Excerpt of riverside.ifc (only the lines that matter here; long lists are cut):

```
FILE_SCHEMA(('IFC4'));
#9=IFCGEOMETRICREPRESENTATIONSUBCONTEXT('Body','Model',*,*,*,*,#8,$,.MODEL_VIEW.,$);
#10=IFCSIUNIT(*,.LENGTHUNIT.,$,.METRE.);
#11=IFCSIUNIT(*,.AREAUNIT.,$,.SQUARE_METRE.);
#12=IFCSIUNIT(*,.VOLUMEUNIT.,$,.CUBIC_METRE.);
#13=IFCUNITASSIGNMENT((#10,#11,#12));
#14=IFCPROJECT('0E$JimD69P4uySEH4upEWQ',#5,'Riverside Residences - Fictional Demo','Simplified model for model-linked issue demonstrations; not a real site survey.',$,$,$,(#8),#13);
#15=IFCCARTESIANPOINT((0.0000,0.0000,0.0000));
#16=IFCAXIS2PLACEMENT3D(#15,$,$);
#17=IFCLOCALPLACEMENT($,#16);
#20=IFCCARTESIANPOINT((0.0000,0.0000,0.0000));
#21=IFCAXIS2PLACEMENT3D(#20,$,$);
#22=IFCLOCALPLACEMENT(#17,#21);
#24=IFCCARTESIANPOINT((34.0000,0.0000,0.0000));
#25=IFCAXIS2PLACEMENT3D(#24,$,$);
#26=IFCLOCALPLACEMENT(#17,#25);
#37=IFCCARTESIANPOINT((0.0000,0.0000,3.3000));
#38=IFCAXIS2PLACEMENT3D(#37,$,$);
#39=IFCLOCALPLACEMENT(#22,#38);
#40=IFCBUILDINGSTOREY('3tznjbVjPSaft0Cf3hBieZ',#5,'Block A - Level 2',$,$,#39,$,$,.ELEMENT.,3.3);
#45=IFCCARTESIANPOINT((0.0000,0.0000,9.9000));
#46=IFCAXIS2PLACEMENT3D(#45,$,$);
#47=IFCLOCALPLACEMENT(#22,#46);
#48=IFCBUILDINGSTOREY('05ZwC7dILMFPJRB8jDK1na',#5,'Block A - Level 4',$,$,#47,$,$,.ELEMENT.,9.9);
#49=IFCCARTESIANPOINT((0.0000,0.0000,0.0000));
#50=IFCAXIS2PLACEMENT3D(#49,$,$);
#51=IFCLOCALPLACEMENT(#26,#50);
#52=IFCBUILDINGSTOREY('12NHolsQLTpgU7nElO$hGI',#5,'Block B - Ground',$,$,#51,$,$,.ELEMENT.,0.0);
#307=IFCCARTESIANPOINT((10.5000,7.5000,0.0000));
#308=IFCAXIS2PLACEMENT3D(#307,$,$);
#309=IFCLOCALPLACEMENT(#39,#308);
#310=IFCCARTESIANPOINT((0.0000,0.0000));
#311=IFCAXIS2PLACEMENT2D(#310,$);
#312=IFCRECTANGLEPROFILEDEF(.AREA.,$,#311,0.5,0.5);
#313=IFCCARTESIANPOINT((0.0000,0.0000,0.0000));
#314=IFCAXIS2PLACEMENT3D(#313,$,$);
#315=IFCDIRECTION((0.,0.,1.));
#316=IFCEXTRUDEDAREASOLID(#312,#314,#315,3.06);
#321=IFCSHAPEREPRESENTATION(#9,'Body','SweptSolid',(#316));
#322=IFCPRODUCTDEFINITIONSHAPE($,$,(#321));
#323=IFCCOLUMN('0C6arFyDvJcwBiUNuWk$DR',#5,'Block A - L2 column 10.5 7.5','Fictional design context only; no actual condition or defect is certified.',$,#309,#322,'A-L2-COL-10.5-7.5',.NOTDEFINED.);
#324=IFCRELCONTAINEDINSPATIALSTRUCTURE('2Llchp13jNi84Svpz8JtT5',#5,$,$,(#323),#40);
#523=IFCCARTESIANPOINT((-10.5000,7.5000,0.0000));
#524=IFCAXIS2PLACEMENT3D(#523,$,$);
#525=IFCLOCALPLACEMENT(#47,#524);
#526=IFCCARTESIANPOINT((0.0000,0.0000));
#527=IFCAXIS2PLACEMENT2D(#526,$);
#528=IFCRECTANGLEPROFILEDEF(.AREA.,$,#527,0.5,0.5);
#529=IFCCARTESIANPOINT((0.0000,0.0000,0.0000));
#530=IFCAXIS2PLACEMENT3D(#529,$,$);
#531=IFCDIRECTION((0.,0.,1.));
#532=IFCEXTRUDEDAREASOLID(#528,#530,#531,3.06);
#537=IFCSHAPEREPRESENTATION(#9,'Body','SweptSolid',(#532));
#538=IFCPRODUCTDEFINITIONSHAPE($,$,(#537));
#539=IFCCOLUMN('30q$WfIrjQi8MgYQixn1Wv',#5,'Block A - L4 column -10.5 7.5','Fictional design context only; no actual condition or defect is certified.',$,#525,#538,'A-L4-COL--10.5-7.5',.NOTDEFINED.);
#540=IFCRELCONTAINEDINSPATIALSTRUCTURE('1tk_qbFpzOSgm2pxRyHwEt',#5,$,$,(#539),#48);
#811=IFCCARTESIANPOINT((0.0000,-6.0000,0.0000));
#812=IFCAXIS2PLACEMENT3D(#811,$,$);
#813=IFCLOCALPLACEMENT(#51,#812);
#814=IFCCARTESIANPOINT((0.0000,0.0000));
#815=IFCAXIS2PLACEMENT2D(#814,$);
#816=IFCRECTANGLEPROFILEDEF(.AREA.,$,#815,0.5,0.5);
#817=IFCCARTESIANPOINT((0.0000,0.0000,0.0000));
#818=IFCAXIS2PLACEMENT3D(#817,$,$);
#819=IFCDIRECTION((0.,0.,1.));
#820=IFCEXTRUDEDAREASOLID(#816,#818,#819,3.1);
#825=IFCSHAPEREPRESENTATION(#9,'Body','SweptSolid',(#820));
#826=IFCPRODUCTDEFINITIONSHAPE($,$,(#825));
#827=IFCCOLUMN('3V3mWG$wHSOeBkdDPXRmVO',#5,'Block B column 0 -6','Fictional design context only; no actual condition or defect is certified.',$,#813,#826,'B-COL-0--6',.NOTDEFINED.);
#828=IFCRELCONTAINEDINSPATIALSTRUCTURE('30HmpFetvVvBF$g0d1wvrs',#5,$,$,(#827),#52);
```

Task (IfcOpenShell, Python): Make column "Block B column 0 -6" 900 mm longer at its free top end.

```python
import ifcopenshell
import ifcopenshell.util.representation

model = ifcopenshell.open("riverside.ifc")

member = model.by_id(827)
change = 0.9

# The extrusion runs towards the end named, so only its depth changes.
body = ifcopenshell.util.representation.get_representation(member, "Model", "Body")
solid = body.Items[0]
old_length = solid.Depth
solid.Depth += change

print(f"length {old_length:g} -> {solid.Depth:g}")

model.write("riverside_updated.ifc")
```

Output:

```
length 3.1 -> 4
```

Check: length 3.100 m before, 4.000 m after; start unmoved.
